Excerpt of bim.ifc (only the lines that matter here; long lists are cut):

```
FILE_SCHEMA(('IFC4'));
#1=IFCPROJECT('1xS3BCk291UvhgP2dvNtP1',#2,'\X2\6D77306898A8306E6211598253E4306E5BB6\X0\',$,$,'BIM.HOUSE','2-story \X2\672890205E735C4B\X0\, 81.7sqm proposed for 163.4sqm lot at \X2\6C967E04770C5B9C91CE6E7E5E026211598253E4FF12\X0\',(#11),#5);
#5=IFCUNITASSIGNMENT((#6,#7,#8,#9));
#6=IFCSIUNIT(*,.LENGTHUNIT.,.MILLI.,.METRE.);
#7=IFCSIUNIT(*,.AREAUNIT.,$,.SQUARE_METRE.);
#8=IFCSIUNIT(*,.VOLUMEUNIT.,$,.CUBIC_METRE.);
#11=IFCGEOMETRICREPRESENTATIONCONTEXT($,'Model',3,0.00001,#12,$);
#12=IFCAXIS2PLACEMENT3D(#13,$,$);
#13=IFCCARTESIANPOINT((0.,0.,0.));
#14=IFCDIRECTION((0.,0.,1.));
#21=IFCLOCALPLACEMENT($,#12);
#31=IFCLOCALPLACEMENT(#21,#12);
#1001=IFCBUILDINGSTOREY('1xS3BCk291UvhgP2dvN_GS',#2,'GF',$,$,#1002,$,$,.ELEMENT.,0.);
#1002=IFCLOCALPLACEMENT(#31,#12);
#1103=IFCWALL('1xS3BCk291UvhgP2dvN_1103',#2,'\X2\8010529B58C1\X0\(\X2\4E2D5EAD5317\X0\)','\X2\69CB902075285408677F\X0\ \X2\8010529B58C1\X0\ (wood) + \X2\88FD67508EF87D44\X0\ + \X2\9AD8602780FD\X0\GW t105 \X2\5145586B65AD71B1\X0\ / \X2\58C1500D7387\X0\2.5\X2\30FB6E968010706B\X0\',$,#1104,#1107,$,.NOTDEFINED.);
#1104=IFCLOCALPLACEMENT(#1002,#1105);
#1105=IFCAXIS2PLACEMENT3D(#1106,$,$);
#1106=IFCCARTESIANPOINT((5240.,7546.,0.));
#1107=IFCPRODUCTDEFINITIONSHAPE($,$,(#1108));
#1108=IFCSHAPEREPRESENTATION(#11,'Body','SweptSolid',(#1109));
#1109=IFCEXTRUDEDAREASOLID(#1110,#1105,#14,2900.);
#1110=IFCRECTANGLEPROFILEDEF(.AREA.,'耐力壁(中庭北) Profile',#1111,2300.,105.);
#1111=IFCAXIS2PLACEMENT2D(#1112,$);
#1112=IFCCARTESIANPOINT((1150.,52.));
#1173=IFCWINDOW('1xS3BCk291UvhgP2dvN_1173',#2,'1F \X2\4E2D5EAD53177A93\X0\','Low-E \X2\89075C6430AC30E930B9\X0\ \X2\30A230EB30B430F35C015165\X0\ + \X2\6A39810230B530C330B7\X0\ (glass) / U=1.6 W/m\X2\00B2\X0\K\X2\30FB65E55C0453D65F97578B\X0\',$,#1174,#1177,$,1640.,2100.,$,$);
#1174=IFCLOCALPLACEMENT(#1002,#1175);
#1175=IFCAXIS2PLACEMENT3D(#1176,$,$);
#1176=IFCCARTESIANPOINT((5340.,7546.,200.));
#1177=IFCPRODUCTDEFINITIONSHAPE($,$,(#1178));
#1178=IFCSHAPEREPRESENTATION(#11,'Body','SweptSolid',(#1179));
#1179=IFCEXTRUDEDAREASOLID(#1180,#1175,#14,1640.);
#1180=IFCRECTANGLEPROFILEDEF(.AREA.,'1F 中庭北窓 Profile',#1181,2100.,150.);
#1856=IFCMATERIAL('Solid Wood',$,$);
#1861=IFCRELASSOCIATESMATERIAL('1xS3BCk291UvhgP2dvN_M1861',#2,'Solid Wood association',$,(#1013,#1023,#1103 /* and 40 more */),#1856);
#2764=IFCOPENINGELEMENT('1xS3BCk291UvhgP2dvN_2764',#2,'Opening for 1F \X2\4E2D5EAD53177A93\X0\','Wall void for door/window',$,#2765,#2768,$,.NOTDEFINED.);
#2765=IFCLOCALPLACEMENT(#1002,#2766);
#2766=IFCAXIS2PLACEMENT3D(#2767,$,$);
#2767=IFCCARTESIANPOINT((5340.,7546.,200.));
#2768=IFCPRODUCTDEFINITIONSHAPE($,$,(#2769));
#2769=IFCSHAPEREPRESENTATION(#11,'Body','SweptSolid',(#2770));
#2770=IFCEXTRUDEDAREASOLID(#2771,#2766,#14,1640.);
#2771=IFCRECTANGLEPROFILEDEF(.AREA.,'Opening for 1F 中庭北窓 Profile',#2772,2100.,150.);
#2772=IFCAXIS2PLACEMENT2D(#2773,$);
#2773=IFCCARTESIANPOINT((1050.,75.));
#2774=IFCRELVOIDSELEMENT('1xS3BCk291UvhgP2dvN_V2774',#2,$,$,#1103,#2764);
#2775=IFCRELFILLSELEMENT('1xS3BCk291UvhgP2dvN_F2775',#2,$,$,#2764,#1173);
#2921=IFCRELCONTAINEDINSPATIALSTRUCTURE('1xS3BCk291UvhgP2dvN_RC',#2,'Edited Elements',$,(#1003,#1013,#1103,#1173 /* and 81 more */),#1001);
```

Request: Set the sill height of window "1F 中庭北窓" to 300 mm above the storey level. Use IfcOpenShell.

```python
import numpy as np
import ifcopenshell
import ifcopenshell.api.geometry
import ifcopenshell.geom
import ifcopenshell.util.element
import ifcopenshell.util.placement
import ifcopenshell.util.shape
import ifcopenshell.util.unit

model = ifcopenshell.open("bim.ifc")
unit_scale = ifcopenshell.util.unit.calculate_unit_scale(model)

window = model.by_guid("1xS3BCk291UvhgP2dvN_1173")
opening = window.FillsVoids[0].RelatingOpeningElement
storey = ifcopenshell.util.element.get_container(window, ifc_class="IfcBuildingStorey")
level = ifcopenshell.util.placement.get_local_placement(storey.ObjectPlacement)[2, 3]

# The opening's origin need not be at the sill, so measure its lowest point.
shape = ifcopenshell.geom.create_shape(ifcopenshell.geom.settings(), opening)
bottom = ifcopenshell.util.shape.get_shape_bottom_elevation(shape, shape.geometry) / unit_scale
dz = level + 300.0 - bottom

shift = np.array([0.0, 0.0, dz])
# The window is not placed relative to its opening, so move both.
for product in (opening, window):
    matrix = ifcopenshell.util.placement.get_local_placement(product.ObjectPlacement)
    matrix[:3, 3] += shift
    ifcopenshell.api.geometry.edit_object_placement(model, product=product, matrix=matrix, is_si=False)

print(f"moved by {dz * unit_scale:+.3f} m")

model.write("bim_v2.ifc")
```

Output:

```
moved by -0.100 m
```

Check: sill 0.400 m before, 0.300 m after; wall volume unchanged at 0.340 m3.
